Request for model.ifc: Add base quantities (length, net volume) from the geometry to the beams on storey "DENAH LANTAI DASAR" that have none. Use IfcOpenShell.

First a look at what the model holds.

```python
import ifcopenshell
import ifcopenshell.util.element
import ifcopenshell.util.unit

model = ifcopenshell.open("model.ifc")
print(model.schema)
for unit_type in ("LENGTHUNIT", "AREAUNIT", "VOLUMEUNIT"):
    print(unit_type, ifcopenshell.util.unit.calculate_unit_scale(model, unit_type))
storey = next(s for s in model.by_type("IfcBuildingStorey") if s.Name == "DENAH LANTAI DASAR")
beams = [e for e in ifcopenshell.util.element.get_decomposition(storey) if e.is_a("IfcBeam")]
for e in sorted(beams, key=lambda e: e.id()):
    print(e.id(), e.is_a(), e.Name, list(ifcopenshell.util.element.get_psets(e, qtos_only=True)), sep=" | ")
```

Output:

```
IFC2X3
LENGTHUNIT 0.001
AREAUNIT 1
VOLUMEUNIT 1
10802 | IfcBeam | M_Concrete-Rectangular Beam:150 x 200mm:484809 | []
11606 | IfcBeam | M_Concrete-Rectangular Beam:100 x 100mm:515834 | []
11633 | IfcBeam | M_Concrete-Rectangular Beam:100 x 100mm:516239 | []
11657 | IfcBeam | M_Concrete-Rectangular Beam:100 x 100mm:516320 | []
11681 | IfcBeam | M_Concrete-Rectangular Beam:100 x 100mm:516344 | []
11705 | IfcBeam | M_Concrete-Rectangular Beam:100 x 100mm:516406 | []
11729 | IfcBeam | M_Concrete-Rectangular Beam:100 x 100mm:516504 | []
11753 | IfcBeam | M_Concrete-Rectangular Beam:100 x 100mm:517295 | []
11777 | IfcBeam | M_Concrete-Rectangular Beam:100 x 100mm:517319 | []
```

```python
import ifcopenshell
import ifcopenshell.api.pset
import ifcopenshell.geom
import ifcopenshell.util.element
import ifcopenshell.util.shape
import ifcopenshell.util.unit

model = ifcopenshell.open("model.ifc")
unit_scale = ifcopenshell.util.unit.calculate_unit_scale(model)
volume_scale = ifcopenshell.util.unit.calculate_unit_scale(model, "VOLUMEUNIT")
settings = ifcopenshell.geom.settings()

storey = next(s for s in model.by_type("IfcBuildingStorey") if s.Name == "DENAH LANTAI DASAR")
beams = [e for e in ifcopenshell.util.element.get_decomposition(storey) if e.is_a("IfcBeam")]

for e in sorted(beams, key=lambda e: e.id()):
    if ifcopenshell.util.element.get_psets(e, qtos_only=True, should_inherit=False):
        continue
    # Geometry comes back in metres, in the element's own axes.
    shape = ifcopenshell.geom.create_shape(settings, e)
    values = {
        "Length": ifcopenshell.util.shape.get_max_xyz(shape.geometry) / unit_scale,
        "NetVolume": ifcopenshell.util.shape.get_volume(shape.geometry) / volume_scale,
    }
    qto = ifcopenshell.api.pset.add_qto(model, product=e, name="BaseQuantities")
    ifcopenshell.api.pset.edit_qto(model, qto=qto, properties=values)
    print(e.id(), {k: round(v, 3) for k, v in values.items()})

model.write("model_rev.ifc")
```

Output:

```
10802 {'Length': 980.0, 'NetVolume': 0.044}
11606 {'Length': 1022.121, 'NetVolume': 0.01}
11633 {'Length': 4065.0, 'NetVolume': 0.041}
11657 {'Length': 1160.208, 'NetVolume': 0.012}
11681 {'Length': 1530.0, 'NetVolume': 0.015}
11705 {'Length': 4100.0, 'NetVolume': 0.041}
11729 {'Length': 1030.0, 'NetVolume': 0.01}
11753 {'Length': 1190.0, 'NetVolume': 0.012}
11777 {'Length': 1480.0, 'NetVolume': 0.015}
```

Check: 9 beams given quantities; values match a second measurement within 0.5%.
